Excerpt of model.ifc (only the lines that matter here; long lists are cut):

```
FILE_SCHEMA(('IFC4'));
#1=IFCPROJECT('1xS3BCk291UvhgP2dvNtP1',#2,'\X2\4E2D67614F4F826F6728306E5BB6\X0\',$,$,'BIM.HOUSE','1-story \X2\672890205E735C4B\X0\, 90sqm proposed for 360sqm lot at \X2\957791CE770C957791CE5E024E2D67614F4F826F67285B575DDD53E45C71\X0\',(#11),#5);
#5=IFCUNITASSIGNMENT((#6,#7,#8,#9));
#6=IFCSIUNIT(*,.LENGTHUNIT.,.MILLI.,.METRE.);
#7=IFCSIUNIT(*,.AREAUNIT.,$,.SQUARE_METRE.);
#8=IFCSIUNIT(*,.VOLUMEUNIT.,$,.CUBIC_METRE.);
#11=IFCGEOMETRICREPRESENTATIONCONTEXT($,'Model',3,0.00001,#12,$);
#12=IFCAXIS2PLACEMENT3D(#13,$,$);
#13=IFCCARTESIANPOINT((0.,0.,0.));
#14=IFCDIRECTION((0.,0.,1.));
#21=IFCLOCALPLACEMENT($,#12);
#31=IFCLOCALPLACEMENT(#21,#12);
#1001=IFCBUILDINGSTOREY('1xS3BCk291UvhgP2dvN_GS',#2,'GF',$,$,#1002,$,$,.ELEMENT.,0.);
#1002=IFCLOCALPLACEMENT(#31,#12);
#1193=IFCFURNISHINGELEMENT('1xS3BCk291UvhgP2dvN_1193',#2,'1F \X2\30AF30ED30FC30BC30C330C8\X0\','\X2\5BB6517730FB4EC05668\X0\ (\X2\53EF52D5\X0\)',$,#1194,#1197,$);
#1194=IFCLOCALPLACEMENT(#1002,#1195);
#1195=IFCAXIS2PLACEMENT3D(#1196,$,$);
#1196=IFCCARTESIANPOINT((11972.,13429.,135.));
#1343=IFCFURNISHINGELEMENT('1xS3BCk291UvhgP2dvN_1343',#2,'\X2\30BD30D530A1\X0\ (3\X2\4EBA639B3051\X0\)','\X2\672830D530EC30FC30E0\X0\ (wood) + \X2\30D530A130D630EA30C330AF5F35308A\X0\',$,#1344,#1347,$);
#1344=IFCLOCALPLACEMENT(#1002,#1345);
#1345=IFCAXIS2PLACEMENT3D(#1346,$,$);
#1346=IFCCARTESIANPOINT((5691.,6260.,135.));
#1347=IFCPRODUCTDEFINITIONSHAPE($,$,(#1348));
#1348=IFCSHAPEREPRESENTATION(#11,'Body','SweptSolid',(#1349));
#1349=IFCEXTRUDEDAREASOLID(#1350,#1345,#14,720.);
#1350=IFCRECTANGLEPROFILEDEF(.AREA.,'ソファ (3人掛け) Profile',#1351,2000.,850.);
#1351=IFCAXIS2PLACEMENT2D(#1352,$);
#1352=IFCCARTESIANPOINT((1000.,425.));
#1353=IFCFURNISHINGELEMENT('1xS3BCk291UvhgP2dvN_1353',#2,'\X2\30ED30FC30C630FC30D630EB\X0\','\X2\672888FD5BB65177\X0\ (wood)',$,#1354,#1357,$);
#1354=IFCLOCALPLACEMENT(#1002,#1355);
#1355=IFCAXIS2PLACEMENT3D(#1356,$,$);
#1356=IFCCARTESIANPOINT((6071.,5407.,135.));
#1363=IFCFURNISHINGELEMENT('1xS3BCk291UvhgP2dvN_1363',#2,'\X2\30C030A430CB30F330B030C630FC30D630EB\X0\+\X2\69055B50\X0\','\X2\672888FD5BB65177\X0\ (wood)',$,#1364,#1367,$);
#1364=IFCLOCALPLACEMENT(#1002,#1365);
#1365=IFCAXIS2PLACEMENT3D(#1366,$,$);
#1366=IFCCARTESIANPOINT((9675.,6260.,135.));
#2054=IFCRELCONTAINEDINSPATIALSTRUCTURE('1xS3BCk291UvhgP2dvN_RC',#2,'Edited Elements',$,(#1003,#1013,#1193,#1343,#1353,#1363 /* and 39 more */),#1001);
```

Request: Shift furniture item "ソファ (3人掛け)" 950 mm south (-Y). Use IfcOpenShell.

```python
import ifcopenshell
import ifcopenshell.api.geometry
import ifcopenshell.util.placement
import ifcopenshell.util.unit

model = ifcopenshell.open("model.ifc")
unit_scale = ifcopenshell.util.unit.calculate_unit_scale(model)

item = model.by_guid("1xS3BCk291UvhgP2dvN_1343")
matrix = ifcopenshell.util.placement.get_local_placement(item.ObjectPlacement)
matrix[1, 3] -= 0.95 / unit_scale
ifcopenshell.api.geometry.edit_object_placement(model, product=item, matrix=matrix, is_si=False)

print(ifcopenshell.util.placement.get_local_placement(item.ObjectPlacement).round(3) + 0.0)

model.write("model_v2.ifc")
```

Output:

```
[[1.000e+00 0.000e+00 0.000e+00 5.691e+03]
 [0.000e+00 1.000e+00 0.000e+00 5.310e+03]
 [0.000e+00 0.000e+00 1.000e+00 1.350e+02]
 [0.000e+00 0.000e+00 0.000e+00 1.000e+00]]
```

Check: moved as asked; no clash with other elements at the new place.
